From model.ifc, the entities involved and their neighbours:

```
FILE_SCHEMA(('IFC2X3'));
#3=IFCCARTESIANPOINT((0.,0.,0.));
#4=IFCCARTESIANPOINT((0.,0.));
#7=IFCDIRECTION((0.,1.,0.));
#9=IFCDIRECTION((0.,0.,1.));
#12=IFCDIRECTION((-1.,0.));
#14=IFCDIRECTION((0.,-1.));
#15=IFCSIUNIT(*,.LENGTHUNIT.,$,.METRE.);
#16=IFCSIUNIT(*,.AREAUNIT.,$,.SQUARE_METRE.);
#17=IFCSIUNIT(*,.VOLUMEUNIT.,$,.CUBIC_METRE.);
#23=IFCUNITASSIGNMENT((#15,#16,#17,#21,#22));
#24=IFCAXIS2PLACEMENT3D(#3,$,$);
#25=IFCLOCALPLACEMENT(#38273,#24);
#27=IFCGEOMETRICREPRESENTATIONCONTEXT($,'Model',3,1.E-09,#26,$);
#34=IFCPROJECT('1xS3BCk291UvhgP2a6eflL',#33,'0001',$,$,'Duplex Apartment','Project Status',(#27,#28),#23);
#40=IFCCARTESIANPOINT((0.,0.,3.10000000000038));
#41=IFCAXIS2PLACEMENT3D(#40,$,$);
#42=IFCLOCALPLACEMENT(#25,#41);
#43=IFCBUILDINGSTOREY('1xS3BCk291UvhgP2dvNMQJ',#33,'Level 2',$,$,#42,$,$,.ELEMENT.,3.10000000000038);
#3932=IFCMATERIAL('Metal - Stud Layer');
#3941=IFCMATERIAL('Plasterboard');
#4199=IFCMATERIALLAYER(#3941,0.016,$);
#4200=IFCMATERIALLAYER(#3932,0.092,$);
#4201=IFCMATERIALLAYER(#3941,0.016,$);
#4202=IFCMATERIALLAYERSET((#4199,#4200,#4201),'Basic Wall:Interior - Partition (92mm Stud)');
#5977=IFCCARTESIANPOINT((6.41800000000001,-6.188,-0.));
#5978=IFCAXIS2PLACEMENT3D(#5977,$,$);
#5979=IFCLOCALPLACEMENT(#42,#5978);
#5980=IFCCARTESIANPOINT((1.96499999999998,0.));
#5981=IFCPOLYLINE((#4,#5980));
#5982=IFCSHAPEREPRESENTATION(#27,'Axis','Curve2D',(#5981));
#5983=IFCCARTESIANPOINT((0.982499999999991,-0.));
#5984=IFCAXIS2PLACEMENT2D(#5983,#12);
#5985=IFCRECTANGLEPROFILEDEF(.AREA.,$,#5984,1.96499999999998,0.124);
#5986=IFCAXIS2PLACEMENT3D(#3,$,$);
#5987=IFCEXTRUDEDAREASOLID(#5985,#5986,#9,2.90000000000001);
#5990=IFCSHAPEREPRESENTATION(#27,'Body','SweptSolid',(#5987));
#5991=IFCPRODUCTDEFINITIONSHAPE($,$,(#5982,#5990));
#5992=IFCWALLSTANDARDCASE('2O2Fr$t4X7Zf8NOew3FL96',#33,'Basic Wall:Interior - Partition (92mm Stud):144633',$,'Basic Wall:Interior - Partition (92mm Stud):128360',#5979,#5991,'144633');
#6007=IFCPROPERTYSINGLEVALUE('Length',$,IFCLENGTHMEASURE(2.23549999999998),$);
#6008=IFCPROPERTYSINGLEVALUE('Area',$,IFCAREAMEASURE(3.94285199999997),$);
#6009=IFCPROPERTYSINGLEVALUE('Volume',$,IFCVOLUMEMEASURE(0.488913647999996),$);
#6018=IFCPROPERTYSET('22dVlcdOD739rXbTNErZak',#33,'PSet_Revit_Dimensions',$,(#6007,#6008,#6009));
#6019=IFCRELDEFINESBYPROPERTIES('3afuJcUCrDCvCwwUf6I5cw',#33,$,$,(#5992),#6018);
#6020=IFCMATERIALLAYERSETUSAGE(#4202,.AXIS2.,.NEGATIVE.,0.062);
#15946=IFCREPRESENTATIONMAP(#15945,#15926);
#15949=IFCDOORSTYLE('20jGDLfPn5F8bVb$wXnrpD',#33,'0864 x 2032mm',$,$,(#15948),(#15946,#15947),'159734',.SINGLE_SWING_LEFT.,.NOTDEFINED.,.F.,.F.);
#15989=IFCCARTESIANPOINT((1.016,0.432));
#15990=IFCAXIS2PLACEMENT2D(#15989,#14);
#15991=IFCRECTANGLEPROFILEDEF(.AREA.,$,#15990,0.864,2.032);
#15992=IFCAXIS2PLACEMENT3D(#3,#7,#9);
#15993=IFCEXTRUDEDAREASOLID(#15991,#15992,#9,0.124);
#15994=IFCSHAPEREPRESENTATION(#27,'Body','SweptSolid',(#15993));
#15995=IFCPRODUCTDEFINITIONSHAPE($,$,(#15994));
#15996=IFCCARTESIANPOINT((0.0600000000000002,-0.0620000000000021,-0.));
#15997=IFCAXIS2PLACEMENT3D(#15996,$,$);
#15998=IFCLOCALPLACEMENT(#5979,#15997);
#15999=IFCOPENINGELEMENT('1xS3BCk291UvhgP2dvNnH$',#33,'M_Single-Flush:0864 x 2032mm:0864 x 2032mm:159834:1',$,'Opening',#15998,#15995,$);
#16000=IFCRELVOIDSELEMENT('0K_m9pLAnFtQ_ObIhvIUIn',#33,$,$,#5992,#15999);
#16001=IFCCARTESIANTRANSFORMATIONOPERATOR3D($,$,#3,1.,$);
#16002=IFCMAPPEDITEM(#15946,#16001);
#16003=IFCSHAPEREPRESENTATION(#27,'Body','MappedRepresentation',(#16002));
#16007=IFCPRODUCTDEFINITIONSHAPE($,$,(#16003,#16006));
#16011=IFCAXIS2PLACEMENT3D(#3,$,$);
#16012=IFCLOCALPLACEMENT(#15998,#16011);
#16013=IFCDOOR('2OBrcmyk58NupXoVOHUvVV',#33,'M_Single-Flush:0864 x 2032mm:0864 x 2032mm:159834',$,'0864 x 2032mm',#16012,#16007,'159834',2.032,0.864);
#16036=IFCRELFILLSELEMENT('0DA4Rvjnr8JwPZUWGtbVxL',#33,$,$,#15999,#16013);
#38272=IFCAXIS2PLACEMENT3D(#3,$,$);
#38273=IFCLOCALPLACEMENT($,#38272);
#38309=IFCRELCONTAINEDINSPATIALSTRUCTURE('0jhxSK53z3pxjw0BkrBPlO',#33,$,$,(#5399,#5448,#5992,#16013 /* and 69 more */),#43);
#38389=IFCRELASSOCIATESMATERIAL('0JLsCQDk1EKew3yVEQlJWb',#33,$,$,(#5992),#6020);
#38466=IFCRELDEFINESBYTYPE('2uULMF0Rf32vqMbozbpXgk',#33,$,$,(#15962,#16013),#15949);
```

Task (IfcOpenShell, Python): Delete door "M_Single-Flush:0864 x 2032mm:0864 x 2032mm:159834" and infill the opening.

```python
import ifcopenshell
import ifcopenshell.api.feature
import ifcopenshell.api.pset
import ifcopenshell.api.root
import ifcopenshell.geom
import ifcopenshell.util.element
import ifcopenshell.util.shape
import ifcopenshell.util.unit

model = ifcopenshell.open("model.ifc")
area_scale = ifcopenshell.util.unit.calculate_unit_scale(model, "AREAUNIT")
volume_scale = ifcopenshell.util.unit.calculate_unit_scale(model, "VOLUMEUNIT")
settings = ifcopenshell.geom.settings()


def volume(element):
    """Net volume in cubic metres, openings subtracted."""
    shape = ifcopenshell.geom.create_shape(settings, element)
    return ifcopenshell.util.shape.get_volume(shape.geometry)


door = model.by_guid("2OBrcmyk58NupXoVOHUvVV")
opening = door.FillsVoids[0].RelatingOpeningElement
wall = opening.VoidsElements[0].RelatingBuildingElement
before = volume(wall)

ifcopenshell.api.root.remove_product(model, product=door)
ifcopenshell.api.feature.remove_feature(model, feature=opening)

after = volume(wall)
thickness = 0.124  # wall thickness in metres

# Update the wall's stored quantities.
pset = model.by_id(ifcopenshell.util.element.get_pset(wall, "PSet_Revit_Dimensions", should_inherit=False)["id"])
ifcopenshell.api.pset.edit_pset(model, pset=pset, properties={
    "Area": model.create_entity("IfcAreaMeasure", after / thickness / area_scale),
    "Volume": model.create_entity("IfcVolumeMeasure", after / volume_scale),
})

print(f"wall volume {before:.3f} -> {after:.3f} m3")

model.write("model_updated.ifc")
```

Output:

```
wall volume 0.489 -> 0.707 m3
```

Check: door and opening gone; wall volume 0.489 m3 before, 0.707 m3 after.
